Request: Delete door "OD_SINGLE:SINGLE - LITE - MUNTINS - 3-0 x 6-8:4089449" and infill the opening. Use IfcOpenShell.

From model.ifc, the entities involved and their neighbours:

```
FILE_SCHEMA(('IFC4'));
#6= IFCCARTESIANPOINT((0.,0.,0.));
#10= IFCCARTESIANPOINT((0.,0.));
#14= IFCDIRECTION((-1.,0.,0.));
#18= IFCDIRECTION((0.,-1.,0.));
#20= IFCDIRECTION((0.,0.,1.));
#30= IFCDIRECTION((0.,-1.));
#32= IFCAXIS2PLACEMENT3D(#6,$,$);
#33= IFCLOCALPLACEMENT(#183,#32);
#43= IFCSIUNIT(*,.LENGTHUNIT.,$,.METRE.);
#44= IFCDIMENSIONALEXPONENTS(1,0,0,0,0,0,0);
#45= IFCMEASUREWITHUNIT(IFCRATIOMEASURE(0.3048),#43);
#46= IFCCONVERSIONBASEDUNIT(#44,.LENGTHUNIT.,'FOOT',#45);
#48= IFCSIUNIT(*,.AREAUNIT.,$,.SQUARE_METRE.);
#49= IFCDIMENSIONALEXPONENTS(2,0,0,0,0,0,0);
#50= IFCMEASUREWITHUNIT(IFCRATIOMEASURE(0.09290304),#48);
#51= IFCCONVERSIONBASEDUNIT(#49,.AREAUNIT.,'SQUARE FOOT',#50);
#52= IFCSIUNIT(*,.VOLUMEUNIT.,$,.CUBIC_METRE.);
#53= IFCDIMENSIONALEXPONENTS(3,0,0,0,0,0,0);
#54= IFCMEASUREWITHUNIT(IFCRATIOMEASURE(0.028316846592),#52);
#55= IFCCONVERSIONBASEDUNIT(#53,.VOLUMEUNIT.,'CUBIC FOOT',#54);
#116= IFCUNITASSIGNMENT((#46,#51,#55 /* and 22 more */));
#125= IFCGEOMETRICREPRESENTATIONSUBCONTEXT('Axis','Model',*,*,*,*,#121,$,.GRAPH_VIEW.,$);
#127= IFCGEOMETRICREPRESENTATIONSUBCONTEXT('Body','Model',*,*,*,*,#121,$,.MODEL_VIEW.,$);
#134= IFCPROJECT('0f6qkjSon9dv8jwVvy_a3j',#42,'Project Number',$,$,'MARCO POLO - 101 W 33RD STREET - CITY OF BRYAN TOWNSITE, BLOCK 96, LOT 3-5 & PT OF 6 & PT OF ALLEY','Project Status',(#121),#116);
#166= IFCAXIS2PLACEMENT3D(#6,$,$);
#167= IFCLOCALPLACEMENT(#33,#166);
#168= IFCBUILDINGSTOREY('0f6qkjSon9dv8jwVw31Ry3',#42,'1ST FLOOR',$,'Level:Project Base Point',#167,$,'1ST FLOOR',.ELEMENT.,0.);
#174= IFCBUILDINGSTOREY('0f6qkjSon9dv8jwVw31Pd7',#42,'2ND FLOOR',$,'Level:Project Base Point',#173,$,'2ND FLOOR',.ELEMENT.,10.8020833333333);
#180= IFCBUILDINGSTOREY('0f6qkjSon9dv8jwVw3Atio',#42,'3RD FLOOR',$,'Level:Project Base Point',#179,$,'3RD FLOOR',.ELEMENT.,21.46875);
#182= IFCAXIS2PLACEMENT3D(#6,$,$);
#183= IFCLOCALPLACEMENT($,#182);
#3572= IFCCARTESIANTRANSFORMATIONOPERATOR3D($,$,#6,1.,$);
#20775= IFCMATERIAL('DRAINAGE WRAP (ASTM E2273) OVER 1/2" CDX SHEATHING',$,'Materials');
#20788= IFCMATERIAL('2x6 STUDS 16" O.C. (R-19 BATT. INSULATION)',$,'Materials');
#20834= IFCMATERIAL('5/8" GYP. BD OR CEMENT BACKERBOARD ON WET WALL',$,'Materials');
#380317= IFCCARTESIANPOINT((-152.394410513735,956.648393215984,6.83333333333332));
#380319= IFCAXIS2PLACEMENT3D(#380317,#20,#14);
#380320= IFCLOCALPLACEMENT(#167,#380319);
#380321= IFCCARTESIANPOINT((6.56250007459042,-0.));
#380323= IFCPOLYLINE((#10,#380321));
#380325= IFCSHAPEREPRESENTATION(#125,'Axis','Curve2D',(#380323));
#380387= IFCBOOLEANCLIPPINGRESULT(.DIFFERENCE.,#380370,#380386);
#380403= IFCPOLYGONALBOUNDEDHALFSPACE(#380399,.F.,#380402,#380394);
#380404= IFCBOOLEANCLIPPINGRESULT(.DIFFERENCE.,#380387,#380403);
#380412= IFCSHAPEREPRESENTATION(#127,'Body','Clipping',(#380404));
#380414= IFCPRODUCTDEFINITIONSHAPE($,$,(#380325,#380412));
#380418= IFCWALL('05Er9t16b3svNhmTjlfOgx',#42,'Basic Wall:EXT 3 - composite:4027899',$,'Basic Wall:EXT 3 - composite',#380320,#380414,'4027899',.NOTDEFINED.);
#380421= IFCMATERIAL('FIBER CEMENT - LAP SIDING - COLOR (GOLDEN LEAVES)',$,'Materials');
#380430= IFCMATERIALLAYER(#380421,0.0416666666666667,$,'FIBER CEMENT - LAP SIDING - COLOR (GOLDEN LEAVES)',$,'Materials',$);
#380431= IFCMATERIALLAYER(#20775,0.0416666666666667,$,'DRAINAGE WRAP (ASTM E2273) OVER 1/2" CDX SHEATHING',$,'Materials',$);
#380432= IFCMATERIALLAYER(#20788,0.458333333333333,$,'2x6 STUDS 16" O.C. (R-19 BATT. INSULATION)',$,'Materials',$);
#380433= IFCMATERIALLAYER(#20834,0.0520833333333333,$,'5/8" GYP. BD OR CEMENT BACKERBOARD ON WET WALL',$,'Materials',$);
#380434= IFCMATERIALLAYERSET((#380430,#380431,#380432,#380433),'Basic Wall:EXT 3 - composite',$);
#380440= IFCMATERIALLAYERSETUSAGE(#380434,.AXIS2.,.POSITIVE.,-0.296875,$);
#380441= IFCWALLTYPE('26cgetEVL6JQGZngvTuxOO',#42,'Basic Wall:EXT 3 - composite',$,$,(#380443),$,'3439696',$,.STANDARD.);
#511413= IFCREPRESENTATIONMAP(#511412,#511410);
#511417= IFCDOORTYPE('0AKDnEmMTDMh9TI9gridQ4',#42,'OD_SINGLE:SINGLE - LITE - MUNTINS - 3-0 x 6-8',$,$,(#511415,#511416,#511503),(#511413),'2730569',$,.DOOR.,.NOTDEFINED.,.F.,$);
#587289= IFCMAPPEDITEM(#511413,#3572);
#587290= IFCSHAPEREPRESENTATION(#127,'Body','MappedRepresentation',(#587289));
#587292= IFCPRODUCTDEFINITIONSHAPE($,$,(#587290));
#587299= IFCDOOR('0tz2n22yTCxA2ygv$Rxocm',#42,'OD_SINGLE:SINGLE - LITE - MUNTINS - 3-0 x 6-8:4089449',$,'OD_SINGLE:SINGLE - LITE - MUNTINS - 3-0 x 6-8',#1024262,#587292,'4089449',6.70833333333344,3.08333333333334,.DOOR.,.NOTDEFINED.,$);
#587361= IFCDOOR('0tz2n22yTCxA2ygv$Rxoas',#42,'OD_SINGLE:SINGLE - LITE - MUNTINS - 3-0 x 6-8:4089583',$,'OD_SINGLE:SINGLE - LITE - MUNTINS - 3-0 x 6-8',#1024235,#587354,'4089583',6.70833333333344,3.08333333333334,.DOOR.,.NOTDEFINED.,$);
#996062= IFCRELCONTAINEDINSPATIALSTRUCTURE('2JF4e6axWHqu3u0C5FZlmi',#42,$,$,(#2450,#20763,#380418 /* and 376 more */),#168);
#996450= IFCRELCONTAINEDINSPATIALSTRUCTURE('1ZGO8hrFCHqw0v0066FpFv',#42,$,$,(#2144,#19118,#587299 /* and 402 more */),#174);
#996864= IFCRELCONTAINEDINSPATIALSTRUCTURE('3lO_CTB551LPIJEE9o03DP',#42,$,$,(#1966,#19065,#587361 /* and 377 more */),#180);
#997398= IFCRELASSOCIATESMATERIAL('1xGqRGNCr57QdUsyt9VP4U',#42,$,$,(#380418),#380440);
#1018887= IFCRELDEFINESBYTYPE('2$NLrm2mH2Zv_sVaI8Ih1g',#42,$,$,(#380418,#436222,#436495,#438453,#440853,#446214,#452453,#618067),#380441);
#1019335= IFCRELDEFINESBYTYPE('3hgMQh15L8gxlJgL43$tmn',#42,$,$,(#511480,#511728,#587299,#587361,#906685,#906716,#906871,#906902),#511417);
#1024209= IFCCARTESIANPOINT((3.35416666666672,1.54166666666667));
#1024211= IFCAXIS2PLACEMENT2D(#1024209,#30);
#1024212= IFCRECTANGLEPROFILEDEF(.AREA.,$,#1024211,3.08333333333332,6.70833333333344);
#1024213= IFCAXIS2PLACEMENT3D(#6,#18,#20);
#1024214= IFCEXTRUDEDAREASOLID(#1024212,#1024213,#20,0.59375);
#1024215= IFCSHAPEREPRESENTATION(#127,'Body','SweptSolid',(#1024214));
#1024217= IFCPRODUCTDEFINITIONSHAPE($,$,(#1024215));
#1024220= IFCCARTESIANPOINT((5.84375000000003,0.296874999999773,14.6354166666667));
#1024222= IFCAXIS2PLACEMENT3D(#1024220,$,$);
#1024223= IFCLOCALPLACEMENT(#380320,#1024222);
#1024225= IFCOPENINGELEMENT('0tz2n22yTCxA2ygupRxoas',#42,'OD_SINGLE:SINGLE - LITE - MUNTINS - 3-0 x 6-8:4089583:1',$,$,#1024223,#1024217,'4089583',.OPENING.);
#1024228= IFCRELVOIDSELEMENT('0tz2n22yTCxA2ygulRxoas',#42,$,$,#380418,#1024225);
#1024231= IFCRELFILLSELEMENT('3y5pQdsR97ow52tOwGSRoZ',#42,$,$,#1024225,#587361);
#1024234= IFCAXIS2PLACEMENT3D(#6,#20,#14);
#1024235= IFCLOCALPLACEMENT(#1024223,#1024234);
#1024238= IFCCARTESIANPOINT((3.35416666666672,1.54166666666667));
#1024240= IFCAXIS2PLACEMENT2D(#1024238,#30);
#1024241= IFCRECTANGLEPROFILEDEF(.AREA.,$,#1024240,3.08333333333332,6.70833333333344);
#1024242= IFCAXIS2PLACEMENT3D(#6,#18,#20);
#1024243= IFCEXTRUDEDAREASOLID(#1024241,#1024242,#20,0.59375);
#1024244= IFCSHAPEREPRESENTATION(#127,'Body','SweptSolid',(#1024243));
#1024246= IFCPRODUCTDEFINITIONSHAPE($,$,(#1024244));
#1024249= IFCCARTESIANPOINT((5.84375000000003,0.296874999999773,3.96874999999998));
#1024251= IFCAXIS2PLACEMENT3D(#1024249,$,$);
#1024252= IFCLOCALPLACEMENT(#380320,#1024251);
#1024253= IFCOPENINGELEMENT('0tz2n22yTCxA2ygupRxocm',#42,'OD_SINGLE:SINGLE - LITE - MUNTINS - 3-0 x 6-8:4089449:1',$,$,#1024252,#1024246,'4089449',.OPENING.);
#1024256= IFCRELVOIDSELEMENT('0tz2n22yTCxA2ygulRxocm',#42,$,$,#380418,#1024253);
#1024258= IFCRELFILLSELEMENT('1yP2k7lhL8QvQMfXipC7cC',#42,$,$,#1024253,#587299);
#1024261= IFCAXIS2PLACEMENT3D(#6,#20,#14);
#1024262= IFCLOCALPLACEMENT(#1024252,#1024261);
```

```python
import ifcopenshell
import ifcopenshell.api.feature
import ifcopenshell.api.root
import ifcopenshell.geom
import ifcopenshell.util.shape

model = ifcopenshell.open("model.ifc")
settings = ifcopenshell.geom.settings()


def volume(element):
    """Net volume in cubic metres, openings subtracted."""
    shape = ifcopenshell.geom.create_shape(settings, element)
    return ifcopenshell.util.shape.get_volume(shape.geometry)


door = model.by_id(587299)
opening = door.FillsVoids[0].RelatingOpeningElement
wall = opening.VoidsElements[0].RelatingBuildingElement
before = volume(wall)

ifcopenshell.api.root.remove_product(model, product=door)
ifcopenshell.api.feature.remove_feature(model, feature=opening)

after = volume(wall)

print(f"wall volume {before:.3f} -> {after:.3f} m3")

model.write("model_v2.ifc")
```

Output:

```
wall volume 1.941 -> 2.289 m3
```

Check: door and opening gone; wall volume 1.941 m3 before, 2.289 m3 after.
